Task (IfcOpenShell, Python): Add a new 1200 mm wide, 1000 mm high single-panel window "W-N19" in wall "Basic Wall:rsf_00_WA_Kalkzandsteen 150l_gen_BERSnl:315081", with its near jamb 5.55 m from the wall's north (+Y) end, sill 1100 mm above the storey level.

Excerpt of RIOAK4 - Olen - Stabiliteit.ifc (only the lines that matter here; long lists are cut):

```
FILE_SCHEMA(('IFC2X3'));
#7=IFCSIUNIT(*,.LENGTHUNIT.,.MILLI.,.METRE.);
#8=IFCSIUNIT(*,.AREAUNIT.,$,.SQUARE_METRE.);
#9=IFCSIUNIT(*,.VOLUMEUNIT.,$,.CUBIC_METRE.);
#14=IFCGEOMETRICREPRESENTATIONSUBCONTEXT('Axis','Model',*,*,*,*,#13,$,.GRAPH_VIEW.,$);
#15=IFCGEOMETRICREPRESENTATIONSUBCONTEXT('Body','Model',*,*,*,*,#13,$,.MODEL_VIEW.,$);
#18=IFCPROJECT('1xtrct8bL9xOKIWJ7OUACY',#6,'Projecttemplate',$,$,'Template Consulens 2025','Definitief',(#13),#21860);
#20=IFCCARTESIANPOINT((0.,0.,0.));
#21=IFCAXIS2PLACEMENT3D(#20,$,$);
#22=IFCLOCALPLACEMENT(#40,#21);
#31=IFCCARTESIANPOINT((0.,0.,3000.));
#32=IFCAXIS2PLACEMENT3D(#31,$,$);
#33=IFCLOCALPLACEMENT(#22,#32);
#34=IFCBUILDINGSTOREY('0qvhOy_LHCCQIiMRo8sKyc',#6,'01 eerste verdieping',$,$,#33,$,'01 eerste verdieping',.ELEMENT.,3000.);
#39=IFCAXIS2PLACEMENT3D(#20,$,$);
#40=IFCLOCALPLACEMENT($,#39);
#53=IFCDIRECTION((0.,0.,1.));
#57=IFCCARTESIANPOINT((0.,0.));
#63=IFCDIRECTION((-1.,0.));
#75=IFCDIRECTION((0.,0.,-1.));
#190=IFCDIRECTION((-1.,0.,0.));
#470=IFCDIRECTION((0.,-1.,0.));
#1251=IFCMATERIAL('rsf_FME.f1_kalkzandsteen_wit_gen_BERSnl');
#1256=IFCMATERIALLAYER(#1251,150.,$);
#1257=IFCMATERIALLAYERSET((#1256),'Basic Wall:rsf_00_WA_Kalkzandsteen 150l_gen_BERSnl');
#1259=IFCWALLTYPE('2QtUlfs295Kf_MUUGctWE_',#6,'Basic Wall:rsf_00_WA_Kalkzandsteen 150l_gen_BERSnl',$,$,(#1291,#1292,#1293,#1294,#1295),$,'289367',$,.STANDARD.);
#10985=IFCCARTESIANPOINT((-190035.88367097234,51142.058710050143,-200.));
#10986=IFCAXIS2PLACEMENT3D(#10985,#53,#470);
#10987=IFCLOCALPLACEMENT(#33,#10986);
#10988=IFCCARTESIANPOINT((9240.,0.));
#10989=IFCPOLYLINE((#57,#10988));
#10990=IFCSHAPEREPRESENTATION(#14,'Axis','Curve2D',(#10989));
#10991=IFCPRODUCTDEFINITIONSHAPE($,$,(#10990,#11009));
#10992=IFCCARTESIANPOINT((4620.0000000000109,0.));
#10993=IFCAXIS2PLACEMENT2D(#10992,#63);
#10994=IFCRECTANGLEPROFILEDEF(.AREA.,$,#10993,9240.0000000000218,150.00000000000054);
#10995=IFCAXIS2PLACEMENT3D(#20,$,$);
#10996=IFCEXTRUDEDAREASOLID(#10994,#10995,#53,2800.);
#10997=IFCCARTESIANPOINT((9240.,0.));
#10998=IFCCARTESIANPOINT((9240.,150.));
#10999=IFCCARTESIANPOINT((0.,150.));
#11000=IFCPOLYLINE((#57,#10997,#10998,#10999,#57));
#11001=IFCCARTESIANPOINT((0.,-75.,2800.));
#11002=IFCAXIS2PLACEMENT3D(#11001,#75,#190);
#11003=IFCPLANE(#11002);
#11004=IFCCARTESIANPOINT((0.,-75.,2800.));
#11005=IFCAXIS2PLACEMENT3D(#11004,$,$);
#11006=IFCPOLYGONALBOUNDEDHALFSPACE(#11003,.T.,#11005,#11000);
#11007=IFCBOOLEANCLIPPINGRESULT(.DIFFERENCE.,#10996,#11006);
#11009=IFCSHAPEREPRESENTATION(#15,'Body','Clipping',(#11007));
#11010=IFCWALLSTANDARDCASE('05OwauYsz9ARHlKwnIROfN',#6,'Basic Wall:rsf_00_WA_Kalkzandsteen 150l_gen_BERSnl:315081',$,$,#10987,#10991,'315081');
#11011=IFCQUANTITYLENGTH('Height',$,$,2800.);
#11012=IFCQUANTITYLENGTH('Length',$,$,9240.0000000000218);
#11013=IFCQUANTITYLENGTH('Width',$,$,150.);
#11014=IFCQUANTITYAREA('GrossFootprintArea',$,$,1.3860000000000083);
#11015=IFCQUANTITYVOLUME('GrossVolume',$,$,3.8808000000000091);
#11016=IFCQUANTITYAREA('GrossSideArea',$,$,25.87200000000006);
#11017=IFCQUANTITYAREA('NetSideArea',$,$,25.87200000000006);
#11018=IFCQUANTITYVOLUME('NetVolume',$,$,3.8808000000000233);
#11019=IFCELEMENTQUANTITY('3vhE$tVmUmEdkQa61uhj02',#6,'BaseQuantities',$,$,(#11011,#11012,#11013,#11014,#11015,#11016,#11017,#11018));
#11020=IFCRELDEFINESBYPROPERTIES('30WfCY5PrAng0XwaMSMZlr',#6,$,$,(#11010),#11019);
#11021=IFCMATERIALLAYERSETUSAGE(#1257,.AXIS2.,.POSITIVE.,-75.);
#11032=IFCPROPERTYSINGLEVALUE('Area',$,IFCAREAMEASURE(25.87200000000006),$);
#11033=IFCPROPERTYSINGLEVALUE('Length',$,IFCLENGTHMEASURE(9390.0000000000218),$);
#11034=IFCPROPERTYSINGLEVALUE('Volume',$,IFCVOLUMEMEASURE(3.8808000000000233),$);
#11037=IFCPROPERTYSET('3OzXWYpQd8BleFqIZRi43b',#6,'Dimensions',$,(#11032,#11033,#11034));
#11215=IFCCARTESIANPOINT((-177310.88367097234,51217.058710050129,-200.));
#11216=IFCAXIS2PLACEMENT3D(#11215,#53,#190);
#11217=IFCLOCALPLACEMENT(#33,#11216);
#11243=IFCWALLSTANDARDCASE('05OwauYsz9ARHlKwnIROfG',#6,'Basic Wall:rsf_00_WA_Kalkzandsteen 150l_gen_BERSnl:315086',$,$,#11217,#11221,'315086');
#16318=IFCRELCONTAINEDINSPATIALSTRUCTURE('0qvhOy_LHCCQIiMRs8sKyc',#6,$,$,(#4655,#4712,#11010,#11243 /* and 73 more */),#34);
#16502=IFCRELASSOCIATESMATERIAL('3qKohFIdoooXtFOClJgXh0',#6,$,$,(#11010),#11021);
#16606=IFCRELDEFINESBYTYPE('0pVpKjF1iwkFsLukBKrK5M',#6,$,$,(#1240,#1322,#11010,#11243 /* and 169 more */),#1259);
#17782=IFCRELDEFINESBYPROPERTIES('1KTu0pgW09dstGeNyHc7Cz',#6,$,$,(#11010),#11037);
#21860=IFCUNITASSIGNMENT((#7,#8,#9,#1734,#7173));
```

```python
import numpy as np
import ifcopenshell
import ifcopenshell.api.feature
import ifcopenshell.api.geometry
import ifcopenshell.api.pset
import ifcopenshell.api.root
import ifcopenshell.api.spatial
import ifcopenshell.api.type
import ifcopenshell.geom
import ifcopenshell.util.element
import ifcopenshell.util.placement
import ifcopenshell.util.representation
import ifcopenshell.util.shape
import ifcopenshell.util.unit

model = ifcopenshell.open("RIOAK4 - Olen - Stabiliteit.ifc")
unit_scale = ifcopenshell.util.unit.calculate_unit_scale(model)
area_scale = ifcopenshell.util.unit.calculate_unit_scale(model, "AREAUNIT")
volume_scale = ifcopenshell.util.unit.calculate_unit_scale(model, "VOLUMEUNIT")
settings = ifcopenshell.geom.settings()


def volume(element):
    """Net volume in cubic metres, openings subtracted."""
    shape = ifcopenshell.geom.create_shape(settings, element)
    return ifcopenshell.util.shape.get_volume(shape.geometry)


wall = model.by_guid("05OwauYsz9ARHlKwnIROfN")
storey = ifcopenshell.util.element.get_container(wall, ifc_class="IfcBuildingStorey")
context = ifcopenshell.util.representation.get_context(model, "Model", "Body", "MODEL_VIEW")
before = volume(wall)

width, height, from_end, sill = 1.2, 1, 5.55, 1.1  # metres

# The wall runs along its own X axis, and the end named is its -X end.
wall_shape = ifcopenshell.geom.create_shape(settings, wall)
x, y, z = ifcopenshell.util.shape.get_vertices(wall_shape.geometry).T
start = x.min() + from_end
face, thickness = float(y.min()), float(y.max() - y.min())
wall_matrix = ifcopenshell.util.placement.get_local_placement(wall.ObjectPlacement)
level = ifcopenshell.util.placement.get_local_placement(storey.ObjectPlacement)[2, 3]


def in_wall(x, y):
    """Placement at x, y metres in the wall's axes, at sill height."""
    matrix = wall_matrix.copy()
    matrix[:, 3] = wall_matrix @ np.array([x / unit_scale, y / unit_scale, 0.0, 1.0])
    matrix[2, 3] = level + sill / unit_scale
    return matrix


# Opening: a box that overshoots both wall faces by 50 mm.
opening = ifcopenshell.api.root.create_entity(model, ifc_class="IfcOpeningElement")
box = ifcopenshell.api.geometry.add_wall_representation(
    model, context=context, length=width, height=height, thickness=thickness + 0.1
)
ifcopenshell.api.geometry.assign_representation(model, product=opening, representation=box)
ifcopenshell.api.geometry.edit_object_placement(model, product=opening, matrix=in_wall(start, face - 0.05), is_si=False)
ifcopenshell.api.feature.add_feature(model, feature=opening, element=wall)

window = ifcopenshell.api.root.create_entity(model, ifc_class="IfcWindow", name="W-N19")
window.OverallWidth, window.OverallHeight = width / unit_scale, height / unit_scale
body = ifcopenshell.api.geometry.add_window_representation(
    model,
    context=context,
    overall_width=window.OverallWidth,
    overall_height=window.OverallHeight,
    partition_type="SINGLE_PANEL",
)
ifcopenshell.api.geometry.assign_representation(model, product=window, representation=body)
ifcopenshell.api.spatial.assign_container(model, products=[window], relating_structure=storey)
fills = ifcopenshell.api.feature.add_filling(model, opening=opening, element=window)
fills.OwnerHistory = window.OwnerHistory  # required in IFC2X3

# IFC2X3 keeps the operation on the window style.
style = ifcopenshell.api.root.create_entity(model, ifc_class="IfcWindowStyle", name="W-N19")
style.OperationType, style.ConstructionType = "SINGLE_PANEL", "NOTDEFINED"
style.ParameterTakesPrecedence = style.Sizeable = False
ifcopenshell.api.type.assign_type(model, related_objects=[window], relating_type=style)

# Centre the window in the wall's thickness.
ifcopenshell.api.geometry.edit_object_placement(model, product=window, matrix=in_wall(start, face), is_si=False)
window_shape = ifcopenshell.geom.create_shape(settings, window)
depth = ifcopenshell.util.shape.get_vertices(window_shape.geometry)[:, 1]
offset = face + thickness / 2 - (depth.min() + depth.max()) / 2
ifcopenshell.api.geometry.edit_object_placement(model, product=window, matrix=in_wall(start, offset), is_si=False)

after = volume(wall)

# Update the wall's stored quantities.
qto = model.by_id(ifcopenshell.util.element.get_pset(wall, "BaseQuantities", should_inherit=False)["id"])
ifcopenshell.api.pset.edit_qto(model, qto=qto, properties={
    "NetSideArea": after / thickness / area_scale,
    "NetVolume": after / volume_scale,
})
pset = model.by_id(ifcopenshell.util.element.get_pset(wall, "Dimensions", should_inherit=False)["id"])
ifcopenshell.api.pset.edit_pset(model, pset=pset, properties={
    "Area": model.create_entity("IfcAreaMeasure", after / thickness / area_scale),
    "Volume": model.create_entity("IfcVolumeMeasure", after / volume_scale),
})

print(f"wall volume {before:.3f} -> {after:.3f} m3")

model.write("RIOAK4 - Olen - Stabiliteit_updated.ifc")
```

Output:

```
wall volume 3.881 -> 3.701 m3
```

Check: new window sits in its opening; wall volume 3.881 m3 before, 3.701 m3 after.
